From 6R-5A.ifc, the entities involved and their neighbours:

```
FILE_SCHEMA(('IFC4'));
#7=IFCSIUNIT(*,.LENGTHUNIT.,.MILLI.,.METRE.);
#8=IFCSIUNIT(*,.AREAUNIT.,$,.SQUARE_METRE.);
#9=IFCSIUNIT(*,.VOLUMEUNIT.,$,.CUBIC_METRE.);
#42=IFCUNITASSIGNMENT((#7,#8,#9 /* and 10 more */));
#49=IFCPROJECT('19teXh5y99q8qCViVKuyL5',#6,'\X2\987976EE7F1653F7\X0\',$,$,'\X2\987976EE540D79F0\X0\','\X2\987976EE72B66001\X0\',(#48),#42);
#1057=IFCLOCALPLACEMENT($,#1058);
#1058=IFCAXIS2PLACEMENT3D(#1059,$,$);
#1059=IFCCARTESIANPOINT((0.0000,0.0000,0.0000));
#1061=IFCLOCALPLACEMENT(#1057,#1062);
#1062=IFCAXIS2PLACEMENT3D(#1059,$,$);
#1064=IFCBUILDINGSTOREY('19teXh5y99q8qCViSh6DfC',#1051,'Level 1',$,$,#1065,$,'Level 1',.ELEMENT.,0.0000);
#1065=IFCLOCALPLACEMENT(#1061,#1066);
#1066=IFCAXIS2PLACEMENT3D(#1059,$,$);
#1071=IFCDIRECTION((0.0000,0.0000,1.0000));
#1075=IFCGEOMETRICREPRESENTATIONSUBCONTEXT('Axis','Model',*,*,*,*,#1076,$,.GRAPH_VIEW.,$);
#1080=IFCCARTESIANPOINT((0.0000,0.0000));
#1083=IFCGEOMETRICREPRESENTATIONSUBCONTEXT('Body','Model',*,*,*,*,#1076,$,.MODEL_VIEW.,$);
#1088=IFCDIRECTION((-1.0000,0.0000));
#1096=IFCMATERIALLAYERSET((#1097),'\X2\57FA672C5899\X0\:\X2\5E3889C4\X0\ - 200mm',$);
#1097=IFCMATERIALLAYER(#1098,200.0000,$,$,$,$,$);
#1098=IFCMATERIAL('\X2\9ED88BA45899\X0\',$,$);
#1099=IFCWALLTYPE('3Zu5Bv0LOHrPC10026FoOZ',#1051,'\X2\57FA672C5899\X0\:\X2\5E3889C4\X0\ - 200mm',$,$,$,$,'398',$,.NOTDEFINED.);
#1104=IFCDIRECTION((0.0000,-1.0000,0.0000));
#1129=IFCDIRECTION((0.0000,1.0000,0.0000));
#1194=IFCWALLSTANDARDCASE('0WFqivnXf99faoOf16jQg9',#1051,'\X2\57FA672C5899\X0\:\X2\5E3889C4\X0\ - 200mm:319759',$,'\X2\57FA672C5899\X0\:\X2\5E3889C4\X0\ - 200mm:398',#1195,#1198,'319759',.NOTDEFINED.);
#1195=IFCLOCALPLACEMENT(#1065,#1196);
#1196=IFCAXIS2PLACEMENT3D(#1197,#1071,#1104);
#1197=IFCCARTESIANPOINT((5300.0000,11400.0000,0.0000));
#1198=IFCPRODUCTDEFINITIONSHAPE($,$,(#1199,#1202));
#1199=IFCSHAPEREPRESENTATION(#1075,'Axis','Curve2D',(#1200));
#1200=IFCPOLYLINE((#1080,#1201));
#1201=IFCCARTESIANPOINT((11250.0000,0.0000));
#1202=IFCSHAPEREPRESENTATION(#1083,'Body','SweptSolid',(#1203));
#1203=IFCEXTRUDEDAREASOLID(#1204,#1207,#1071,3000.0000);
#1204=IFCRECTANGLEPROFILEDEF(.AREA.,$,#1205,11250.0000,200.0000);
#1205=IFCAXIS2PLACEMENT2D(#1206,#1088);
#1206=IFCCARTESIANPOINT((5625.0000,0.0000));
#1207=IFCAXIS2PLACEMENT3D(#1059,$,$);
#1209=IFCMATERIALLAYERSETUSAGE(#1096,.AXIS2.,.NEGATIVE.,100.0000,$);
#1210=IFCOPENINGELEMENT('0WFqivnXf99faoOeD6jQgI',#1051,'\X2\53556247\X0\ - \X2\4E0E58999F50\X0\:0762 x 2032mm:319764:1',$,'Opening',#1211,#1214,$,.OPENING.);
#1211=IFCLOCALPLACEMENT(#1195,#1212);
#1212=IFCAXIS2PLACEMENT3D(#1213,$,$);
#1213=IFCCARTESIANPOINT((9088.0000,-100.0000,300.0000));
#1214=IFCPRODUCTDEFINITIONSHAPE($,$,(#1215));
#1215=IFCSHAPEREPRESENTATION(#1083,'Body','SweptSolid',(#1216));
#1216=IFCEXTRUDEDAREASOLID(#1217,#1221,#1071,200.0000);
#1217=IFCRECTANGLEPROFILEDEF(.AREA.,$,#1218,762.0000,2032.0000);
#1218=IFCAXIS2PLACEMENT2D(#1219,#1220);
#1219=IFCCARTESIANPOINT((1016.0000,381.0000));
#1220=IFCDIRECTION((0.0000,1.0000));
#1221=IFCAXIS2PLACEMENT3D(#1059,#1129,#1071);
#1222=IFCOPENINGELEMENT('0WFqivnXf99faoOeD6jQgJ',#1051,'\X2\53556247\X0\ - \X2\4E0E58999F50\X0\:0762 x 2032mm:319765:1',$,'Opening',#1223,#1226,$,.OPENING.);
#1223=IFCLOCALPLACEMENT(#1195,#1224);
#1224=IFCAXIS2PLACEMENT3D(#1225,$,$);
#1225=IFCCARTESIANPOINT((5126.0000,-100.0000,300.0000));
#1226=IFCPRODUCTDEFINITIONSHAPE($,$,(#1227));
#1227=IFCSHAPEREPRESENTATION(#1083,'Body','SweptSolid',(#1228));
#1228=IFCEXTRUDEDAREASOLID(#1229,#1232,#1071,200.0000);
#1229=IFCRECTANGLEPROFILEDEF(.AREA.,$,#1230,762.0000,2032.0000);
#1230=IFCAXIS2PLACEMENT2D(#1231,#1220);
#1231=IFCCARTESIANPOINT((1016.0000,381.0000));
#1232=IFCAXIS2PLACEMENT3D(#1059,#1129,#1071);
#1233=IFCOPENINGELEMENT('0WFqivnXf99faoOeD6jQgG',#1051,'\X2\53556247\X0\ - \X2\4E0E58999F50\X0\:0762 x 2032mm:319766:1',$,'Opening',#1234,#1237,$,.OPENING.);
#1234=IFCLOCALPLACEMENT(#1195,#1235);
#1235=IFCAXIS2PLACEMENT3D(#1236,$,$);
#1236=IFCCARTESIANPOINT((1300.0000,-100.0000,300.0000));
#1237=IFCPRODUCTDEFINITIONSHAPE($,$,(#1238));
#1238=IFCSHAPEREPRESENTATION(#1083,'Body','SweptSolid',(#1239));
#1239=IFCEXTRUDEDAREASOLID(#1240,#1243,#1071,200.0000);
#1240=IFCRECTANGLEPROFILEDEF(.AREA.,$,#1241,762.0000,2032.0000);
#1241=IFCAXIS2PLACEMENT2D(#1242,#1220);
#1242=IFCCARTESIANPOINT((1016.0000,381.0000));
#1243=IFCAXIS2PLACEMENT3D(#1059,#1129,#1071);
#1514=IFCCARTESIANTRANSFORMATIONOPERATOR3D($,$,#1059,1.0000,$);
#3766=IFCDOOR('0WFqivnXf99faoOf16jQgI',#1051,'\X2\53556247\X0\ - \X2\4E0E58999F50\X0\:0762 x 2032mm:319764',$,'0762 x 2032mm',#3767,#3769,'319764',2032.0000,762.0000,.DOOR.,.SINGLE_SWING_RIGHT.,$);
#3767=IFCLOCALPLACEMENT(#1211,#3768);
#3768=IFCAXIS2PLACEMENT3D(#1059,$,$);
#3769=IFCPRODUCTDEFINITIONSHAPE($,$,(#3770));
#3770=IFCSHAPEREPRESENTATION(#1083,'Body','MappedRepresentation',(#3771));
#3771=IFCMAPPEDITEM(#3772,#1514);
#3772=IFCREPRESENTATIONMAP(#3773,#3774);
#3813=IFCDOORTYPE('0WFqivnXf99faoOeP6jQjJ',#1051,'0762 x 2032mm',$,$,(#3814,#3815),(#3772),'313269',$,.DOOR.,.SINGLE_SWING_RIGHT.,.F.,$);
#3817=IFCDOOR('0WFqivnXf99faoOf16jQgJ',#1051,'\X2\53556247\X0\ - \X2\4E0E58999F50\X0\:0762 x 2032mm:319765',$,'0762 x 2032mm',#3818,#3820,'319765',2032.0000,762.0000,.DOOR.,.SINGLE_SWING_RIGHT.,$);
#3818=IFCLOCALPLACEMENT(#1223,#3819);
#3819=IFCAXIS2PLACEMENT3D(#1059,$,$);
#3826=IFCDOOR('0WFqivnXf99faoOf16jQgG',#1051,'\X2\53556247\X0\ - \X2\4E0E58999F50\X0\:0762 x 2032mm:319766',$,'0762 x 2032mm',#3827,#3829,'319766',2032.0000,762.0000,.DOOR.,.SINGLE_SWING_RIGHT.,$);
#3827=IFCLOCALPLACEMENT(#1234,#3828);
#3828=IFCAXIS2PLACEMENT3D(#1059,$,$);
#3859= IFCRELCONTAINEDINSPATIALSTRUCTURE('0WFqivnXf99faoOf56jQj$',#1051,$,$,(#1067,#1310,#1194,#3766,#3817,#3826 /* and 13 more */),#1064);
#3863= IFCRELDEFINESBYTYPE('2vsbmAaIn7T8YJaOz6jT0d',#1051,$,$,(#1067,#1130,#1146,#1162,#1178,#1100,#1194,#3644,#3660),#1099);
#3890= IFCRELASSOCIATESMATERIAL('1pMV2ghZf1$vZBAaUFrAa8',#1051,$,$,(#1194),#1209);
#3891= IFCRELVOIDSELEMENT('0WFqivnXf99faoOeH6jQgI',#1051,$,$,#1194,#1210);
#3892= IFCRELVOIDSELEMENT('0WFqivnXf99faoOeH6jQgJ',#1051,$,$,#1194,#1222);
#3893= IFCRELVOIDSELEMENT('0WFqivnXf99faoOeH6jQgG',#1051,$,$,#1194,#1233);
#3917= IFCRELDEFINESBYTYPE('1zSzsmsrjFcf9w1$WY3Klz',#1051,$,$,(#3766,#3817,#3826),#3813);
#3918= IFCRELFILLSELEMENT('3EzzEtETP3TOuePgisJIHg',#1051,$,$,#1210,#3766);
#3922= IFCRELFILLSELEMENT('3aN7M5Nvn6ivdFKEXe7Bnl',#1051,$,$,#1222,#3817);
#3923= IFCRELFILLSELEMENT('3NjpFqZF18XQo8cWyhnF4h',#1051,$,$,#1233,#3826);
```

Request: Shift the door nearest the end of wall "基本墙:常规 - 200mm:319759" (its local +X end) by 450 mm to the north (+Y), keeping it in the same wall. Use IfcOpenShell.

```python
import ifcopenshell
import ifcopenshell.api.geometry
import ifcopenshell.util.placement
import ifcopenshell.util.unit

model = ifcopenshell.open("6R-5A.ifc")
unit_scale = ifcopenshell.util.unit.calculate_unit_scale(model)

door = model.by_id(3766)
opening = door.FillsVoids[0].RelatingOpeningElement
wall = opening.VoidsElements[0].RelatingBuildingElement

wall_matrix = ifcopenshell.util.placement.get_local_placement(wall.ObjectPlacement)
shift = wall_matrix[:3, 0] * -0.45 / unit_scale
before = ifcopenshell.util.placement.get_local_placement(door.ObjectPlacement)[:3, 3].copy()

# The door is placed relative to its opening, so it follows when the opening moves.
matrix = ifcopenshell.util.placement.get_local_placement(opening.ObjectPlacement)
matrix[:3, 3] += shift
ifcopenshell.api.geometry.edit_object_placement(
    model, product=opening, matrix=matrix, is_si=False, should_transform_children=True
)

after = ifcopenshell.util.placement.get_local_placement(door.ObjectPlacement)[:3, 3]
print("door moved by", (after - before).round(3) + 0.0)

model.write("6R-5A_v2.ifc")
```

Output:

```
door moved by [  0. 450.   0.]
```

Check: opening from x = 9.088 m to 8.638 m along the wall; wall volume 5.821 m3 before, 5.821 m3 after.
